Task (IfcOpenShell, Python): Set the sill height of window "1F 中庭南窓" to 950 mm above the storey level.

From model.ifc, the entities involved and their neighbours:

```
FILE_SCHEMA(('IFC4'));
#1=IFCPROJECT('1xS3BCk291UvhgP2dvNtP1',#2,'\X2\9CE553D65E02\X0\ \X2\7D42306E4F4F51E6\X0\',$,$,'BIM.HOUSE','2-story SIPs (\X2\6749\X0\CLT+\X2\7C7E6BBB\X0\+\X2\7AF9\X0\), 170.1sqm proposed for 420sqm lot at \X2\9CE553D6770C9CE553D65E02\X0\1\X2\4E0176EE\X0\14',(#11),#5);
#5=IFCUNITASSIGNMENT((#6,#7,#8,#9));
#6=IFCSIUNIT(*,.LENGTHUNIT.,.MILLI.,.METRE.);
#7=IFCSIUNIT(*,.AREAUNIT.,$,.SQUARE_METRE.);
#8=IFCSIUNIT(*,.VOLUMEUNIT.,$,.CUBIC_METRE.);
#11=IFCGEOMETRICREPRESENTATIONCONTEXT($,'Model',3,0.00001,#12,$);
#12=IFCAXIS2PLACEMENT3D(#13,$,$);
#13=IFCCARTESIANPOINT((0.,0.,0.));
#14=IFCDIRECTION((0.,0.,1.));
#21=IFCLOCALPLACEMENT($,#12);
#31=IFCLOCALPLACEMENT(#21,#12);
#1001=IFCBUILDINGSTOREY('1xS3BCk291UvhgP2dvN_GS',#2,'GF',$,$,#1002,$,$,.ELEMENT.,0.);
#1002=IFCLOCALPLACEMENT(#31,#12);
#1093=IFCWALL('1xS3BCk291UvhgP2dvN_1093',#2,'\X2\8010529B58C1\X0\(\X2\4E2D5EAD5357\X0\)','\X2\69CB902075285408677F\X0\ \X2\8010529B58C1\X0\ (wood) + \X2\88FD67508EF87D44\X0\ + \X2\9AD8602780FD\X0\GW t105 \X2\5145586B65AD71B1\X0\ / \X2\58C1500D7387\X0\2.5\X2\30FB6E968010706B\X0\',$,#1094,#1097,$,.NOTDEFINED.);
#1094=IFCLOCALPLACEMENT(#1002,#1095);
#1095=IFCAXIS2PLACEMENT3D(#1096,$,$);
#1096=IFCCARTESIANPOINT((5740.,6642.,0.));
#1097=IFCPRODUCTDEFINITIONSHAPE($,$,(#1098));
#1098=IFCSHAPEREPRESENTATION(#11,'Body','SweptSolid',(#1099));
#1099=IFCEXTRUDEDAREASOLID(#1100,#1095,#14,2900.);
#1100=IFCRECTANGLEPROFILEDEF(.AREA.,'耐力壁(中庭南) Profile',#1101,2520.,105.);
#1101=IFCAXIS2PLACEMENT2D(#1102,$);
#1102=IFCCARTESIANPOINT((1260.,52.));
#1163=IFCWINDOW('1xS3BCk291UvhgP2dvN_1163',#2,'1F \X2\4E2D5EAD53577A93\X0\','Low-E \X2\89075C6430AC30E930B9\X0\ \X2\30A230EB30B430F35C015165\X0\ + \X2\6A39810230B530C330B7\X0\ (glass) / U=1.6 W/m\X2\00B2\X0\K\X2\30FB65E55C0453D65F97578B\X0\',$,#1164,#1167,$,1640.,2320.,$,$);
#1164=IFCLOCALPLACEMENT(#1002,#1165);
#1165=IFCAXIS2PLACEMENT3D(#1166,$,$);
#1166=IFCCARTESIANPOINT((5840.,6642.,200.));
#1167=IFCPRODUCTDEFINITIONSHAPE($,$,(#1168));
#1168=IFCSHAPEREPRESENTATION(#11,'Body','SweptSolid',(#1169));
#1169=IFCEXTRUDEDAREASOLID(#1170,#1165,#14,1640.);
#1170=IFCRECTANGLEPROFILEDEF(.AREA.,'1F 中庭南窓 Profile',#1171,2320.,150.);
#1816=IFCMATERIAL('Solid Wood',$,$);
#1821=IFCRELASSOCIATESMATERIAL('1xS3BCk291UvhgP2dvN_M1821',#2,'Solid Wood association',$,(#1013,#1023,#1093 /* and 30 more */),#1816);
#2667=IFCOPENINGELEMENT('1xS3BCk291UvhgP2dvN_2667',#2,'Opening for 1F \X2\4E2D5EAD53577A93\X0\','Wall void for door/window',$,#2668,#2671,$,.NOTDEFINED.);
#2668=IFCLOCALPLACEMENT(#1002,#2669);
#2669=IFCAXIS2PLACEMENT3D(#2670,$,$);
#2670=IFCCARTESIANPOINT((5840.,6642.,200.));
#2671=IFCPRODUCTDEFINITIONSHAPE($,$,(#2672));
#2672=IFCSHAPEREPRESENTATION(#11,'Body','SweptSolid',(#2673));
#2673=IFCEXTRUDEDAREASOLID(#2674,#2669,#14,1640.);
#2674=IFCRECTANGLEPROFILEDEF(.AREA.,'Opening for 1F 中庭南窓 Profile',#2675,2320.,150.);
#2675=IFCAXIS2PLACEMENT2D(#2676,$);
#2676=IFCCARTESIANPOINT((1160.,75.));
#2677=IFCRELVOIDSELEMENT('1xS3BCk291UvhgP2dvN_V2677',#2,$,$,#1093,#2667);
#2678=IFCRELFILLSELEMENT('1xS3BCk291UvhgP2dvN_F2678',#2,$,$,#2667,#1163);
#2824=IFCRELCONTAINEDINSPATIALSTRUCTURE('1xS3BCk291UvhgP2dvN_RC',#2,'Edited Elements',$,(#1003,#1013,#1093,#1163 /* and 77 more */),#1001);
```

```python
import numpy as np
import ifcopenshell
import ifcopenshell.api.geometry
import ifcopenshell.geom
import ifcopenshell.util.element
import ifcopenshell.util.placement
import ifcopenshell.util.shape
import ifcopenshell.util.unit

model = ifcopenshell.open("model.ifc")
unit_scale = ifcopenshell.util.unit.calculate_unit_scale(model)

window = model.by_id(1163)
opening = window.FillsVoids[0].RelatingOpeningElement
storey = ifcopenshell.util.element.get_container(window, ifc_class="IfcBuildingStorey")
level = ifcopenshell.util.placement.get_local_placement(storey.ObjectPlacement)[2, 3]

# The opening's origin need not be at the sill, so measure its lowest point.
shape = ifcopenshell.geom.create_shape(ifcopenshell.geom.settings(), opening)
bottom = ifcopenshell.util.shape.get_shape_bottom_elevation(shape, shape.geometry) / unit_scale
dz = level + 950.0 - bottom

shift = np.array([0.0, 0.0, dz])
# The window is not placed relative to its opening, so move both.
for product in (opening, window):
    matrix = ifcopenshell.util.placement.get_local_placement(product.ObjectPlacement)
    matrix[:3, 3] += shift
    ifcopenshell.api.geometry.edit_object_placement(model, product=product, matrix=matrix, is_si=False)

print(f"moved by {dz * unit_scale:+.3f} m")

model.write("model-out.ifc")
```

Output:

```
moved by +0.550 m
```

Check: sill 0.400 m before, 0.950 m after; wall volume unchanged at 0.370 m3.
